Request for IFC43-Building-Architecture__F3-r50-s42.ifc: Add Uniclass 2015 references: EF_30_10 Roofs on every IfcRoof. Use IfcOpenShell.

First a look at what the model holds.

```python
import ifcopenshell

model = ifcopenshell.open("IFC43-Building-Architecture__F3-r50-s42.ifc")
print(model.schema)
print("classifications:", [c.Name for c in model.by_type("IfcClassification")])
for ifc_class in ("IfcDoor", "IfcRoof", "IfcStair", "IfcWall", "IfcWindow"):
    print(ifc_class, len(model.by_type(ifc_class)))
```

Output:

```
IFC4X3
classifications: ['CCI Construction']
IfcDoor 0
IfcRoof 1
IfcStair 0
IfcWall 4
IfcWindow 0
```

```python
import ifcopenshell
import ifcopenshell.api.classification

model = ifcopenshell.open("IFC43-Building-Architecture__F3-r50-s42.ifc")

system = ifcopenshell.api.classification.add_classification(model, classification="Uniclass 2015")

codes = {
    "IfcRoof": ("EF_30_10", "Roofs"),
}
for ifc_class, (code, name) in codes.items():
    products = model.by_type(ifc_class)
    ifcopenshell.api.classification.add_reference(
        model, products=products, classification=system, identification=code, name=name
    )
    print(code, len(products))

model.write("IFC43-Building-Architecture__F3-r50-s42_rev.ifc")
```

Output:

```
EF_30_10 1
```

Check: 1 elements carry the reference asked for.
